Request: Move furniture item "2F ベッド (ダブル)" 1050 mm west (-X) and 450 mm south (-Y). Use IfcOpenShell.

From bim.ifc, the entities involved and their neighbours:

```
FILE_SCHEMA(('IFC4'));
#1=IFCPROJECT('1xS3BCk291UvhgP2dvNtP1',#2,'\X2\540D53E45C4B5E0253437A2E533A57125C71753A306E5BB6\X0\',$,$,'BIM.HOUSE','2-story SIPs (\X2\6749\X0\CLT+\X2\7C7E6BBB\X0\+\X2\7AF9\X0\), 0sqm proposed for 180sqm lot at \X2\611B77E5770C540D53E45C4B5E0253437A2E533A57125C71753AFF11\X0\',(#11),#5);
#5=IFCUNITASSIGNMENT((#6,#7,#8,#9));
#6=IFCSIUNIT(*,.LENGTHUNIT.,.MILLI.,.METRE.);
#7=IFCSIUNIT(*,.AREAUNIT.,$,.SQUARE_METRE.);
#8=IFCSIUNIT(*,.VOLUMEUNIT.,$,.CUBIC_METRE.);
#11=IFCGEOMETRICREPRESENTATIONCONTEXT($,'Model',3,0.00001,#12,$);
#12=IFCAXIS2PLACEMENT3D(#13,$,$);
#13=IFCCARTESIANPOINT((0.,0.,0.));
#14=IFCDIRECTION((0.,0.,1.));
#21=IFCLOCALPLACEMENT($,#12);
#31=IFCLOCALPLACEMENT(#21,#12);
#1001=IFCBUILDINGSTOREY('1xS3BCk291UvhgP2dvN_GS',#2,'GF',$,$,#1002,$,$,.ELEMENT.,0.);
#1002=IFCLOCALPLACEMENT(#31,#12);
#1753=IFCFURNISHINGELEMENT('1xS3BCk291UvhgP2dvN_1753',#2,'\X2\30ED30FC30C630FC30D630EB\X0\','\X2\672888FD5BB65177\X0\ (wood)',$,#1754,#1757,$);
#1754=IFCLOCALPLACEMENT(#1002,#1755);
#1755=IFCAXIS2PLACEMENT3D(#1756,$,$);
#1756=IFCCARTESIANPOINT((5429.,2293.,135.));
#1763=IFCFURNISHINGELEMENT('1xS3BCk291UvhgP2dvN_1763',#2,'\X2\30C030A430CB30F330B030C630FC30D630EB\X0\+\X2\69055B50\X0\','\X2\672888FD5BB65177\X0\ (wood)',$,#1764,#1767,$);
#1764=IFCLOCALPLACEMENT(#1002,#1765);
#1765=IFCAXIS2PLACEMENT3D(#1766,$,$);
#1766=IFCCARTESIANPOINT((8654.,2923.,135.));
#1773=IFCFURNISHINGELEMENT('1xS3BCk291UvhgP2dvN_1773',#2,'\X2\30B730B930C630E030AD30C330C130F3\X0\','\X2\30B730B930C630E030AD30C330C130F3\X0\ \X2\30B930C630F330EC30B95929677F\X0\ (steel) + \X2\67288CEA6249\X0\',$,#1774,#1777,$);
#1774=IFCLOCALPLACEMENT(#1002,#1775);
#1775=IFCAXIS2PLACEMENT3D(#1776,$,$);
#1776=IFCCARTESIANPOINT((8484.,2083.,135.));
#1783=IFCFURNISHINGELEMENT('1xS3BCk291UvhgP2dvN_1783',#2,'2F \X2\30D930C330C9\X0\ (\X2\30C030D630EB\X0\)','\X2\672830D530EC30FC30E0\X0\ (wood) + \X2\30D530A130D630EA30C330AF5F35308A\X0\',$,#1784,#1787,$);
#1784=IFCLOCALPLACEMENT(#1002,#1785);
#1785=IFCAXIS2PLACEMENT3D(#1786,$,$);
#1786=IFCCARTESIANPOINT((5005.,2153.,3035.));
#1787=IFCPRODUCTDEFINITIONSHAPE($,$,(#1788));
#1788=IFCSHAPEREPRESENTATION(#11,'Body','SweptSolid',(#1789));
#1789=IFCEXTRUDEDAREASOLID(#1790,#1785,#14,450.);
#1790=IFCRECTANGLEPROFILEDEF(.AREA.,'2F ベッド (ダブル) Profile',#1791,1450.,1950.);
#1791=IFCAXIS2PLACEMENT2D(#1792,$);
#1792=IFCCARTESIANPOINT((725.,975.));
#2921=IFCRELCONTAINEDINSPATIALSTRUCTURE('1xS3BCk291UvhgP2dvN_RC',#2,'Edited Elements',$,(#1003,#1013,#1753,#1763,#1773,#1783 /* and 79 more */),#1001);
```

```python
import ifcopenshell
import ifcopenshell.api.geometry
import ifcopenshell.util.placement
import ifcopenshell.util.unit

model = ifcopenshell.open("bim.ifc")
unit_scale = ifcopenshell.util.unit.calculate_unit_scale(model)

item = model.by_guid("1xS3BCk291UvhgP2dvN_1783")
matrix = ifcopenshell.util.placement.get_local_placement(item.ObjectPlacement)
matrix[0, 3] -= 1.05 / unit_scale
matrix[1, 3] -= 0.45 / unit_scale
ifcopenshell.api.geometry.edit_object_placement(model, product=item, matrix=matrix, is_si=False)

print(ifcopenshell.util.placement.get_local_placement(item.ObjectPlacement).round(3) + 0.0)

model.write("bim_edited.ifc")
```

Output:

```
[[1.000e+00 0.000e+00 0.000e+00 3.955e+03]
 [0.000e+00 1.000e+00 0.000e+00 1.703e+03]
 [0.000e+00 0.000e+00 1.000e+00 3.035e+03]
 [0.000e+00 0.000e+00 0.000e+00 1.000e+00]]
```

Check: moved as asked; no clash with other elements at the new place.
